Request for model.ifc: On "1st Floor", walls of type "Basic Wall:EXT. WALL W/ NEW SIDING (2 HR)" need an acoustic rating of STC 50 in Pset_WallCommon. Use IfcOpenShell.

First a look at what the model holds.

```python
import ifcopenshell
import ifcopenshell.util.element

model = ifcopenshell.open("model.ifc")
print(model.schema)
storey = next(s for s in model.by_type("IfcBuildingStorey") if s.Name == "1st Floor")
walls = [e for e in ifcopenshell.util.element.get_decomposition(storey) if e.is_a("IfcWall")]
seen = {}
for e in walls:
    element_type = ifcopenshell.util.element.get_type(e)
    key = (element_type.Name if element_type != e and element_type else None, ifcopenshell.util.element.get_pset(e, "Pset_WallCommon", "AcousticRating"))
    seen[key] = seen.get(key, 0) + 1
for (name, value), count in sorted(seen.items(), key=str):
    print(count, "x", name, "|", value)
```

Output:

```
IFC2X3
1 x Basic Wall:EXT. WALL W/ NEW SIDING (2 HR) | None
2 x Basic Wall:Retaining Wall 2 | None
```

```python
import ifcopenshell
import ifcopenshell.api.pset
import ifcopenshell.util.element

model = ifcopenshell.open("model.ifc")

storey = next(s for s in model.by_type("IfcBuildingStorey") if s.Name == "1st Floor")
walls = [e for e in ifcopenshell.util.element.get_decomposition(storey) if e.is_a("IfcWall")]

count = 0
for e in walls:
    element_type = ifcopenshell.util.element.get_type(e)
    if element_type in (None, e) or element_type.Name != "Basic Wall:EXT. WALL W/ NEW SIDING (2 HR)":
        continue
    # add_pset returns the element's existing set when there is one.
    pset = ifcopenshell.api.pset.add_pset(model, product=e, name="Pset_WallCommon")
    ifcopenshell.api.pset.edit_pset(model, pset=pset, properties={"AcousticRating": "STC 50"})
    count += 1

print(count, "walls updated")

model.write("model_rev.ifc")
```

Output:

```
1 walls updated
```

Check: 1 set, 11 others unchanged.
